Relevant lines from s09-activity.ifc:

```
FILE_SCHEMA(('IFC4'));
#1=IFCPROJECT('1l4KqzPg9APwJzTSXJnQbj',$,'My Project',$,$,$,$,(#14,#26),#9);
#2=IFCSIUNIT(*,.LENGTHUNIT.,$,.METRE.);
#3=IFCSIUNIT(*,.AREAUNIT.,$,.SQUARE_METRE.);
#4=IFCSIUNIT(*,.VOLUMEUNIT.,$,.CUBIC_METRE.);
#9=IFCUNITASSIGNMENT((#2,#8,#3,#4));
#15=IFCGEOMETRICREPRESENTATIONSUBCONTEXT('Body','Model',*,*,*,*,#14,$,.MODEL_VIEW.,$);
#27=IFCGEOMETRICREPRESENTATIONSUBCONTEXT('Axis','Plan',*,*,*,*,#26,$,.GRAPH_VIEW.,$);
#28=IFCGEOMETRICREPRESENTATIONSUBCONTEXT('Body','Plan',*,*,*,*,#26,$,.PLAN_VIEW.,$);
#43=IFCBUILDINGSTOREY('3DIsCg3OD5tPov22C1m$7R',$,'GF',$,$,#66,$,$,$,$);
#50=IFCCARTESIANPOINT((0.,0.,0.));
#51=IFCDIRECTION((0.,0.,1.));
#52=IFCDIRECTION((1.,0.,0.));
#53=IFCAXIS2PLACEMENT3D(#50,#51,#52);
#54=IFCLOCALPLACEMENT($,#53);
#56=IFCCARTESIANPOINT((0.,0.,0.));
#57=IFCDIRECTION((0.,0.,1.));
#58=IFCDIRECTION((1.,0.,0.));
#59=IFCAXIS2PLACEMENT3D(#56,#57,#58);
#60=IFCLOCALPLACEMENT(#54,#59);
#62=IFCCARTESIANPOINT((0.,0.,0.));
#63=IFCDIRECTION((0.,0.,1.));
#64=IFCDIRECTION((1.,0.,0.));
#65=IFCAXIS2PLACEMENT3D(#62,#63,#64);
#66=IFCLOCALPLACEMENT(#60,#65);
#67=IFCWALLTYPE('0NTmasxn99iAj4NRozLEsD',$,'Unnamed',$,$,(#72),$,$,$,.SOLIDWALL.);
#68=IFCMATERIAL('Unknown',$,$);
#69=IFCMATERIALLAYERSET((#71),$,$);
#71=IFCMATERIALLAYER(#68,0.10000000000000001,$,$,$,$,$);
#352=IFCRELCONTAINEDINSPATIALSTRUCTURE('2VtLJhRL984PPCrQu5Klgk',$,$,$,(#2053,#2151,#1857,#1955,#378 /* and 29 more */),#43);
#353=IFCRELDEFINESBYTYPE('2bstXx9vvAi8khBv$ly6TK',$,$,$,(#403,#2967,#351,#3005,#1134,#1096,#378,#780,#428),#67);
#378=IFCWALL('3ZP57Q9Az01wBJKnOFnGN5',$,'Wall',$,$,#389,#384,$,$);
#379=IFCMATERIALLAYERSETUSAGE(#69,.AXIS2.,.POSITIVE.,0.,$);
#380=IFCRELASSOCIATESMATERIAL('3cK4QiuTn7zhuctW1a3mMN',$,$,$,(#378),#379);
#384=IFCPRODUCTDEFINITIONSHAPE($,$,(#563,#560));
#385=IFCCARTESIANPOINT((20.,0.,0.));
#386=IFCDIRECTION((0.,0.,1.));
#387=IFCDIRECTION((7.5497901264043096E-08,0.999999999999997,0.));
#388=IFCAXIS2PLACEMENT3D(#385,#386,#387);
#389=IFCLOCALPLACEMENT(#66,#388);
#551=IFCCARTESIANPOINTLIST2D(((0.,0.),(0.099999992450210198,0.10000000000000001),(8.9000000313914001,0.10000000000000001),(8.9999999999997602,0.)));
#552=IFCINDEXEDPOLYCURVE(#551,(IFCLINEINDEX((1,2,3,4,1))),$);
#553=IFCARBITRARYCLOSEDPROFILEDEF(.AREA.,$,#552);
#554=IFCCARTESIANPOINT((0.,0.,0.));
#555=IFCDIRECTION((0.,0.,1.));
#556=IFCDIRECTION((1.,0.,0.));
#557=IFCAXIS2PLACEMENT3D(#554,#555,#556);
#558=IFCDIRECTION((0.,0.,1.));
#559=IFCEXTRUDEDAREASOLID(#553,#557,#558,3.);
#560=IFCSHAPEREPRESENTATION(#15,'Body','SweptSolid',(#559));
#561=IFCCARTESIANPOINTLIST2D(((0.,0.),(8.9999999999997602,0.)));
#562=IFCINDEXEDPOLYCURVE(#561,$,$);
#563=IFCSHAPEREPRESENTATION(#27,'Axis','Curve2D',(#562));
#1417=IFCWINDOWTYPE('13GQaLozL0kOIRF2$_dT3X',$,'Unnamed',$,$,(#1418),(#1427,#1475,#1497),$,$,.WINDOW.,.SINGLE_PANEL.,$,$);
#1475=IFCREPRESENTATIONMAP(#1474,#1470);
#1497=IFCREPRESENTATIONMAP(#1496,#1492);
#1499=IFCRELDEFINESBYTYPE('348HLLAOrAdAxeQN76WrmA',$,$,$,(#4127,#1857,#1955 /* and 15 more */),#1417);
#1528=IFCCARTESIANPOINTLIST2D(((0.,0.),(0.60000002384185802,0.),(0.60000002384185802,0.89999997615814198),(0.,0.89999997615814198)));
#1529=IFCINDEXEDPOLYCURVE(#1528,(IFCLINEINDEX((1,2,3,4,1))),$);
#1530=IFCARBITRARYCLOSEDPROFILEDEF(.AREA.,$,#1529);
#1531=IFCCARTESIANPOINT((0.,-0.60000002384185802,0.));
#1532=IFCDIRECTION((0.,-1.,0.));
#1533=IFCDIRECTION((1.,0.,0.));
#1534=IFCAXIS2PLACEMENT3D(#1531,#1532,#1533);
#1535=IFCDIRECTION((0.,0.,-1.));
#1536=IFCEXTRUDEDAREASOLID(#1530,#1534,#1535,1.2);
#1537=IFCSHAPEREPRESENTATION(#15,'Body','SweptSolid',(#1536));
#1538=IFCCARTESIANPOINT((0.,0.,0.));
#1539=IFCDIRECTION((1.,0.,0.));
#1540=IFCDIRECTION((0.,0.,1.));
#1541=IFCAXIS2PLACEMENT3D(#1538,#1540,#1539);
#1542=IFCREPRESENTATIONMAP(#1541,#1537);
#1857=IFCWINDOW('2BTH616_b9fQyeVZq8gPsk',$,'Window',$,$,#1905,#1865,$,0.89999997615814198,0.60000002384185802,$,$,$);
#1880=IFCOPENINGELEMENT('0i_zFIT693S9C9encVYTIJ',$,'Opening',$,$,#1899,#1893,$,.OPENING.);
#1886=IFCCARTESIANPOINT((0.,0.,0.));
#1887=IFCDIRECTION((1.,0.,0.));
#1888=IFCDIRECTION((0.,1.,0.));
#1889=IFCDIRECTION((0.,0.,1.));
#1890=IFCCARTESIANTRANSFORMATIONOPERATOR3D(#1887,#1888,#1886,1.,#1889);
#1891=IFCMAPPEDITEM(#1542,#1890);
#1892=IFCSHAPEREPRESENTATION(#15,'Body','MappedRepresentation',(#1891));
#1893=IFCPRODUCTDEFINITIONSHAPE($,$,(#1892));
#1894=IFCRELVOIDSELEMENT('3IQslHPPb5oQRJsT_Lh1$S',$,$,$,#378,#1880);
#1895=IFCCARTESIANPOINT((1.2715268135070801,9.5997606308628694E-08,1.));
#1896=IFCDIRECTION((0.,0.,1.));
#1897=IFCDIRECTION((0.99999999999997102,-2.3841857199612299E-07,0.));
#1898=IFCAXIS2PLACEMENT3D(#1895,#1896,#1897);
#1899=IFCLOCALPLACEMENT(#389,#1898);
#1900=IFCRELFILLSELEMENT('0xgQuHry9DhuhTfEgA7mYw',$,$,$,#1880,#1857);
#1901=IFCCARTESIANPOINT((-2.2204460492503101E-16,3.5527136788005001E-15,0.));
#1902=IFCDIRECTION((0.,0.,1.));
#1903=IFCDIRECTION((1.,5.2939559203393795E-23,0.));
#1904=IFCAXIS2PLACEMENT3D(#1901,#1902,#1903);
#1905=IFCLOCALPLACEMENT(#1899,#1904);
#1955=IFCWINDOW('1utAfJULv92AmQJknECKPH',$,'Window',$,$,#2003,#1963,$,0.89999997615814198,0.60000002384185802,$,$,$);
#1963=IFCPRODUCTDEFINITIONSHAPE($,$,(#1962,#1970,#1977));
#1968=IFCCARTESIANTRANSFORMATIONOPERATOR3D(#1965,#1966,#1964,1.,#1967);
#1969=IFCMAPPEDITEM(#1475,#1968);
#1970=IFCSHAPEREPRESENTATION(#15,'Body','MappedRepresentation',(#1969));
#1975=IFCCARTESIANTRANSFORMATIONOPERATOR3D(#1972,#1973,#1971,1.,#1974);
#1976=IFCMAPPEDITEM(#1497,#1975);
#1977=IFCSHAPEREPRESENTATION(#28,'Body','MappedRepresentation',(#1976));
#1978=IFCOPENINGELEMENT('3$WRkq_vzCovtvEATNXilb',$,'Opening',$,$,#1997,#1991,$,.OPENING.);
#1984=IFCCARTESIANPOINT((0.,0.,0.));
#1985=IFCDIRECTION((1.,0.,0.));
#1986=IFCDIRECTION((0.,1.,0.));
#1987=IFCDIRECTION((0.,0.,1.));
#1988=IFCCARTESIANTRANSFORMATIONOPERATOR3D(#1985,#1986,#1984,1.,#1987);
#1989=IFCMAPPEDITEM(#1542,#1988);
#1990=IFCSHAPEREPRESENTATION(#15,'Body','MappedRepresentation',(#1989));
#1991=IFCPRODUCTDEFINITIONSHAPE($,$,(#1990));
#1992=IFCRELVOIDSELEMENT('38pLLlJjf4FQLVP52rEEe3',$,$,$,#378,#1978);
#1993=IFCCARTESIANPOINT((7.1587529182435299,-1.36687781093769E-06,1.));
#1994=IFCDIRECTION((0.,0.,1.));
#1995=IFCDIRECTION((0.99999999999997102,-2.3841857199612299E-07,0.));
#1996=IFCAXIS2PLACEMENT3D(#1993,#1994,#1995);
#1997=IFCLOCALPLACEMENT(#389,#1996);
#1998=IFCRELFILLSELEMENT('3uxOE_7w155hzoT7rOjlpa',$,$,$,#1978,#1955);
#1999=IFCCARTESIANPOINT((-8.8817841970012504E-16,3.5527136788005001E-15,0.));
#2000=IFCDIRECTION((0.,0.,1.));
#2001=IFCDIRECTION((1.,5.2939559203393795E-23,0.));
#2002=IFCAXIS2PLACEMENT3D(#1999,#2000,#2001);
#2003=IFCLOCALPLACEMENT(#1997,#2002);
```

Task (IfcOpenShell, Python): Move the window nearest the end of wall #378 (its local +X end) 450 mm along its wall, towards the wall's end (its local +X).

```python
import ifcopenshell
import ifcopenshell.api.geometry
import ifcopenshell.util.placement

model = ifcopenshell.open("s09-activity.ifc")

window = model.by_guid("1utAfJULv92AmQJknECKPH")
opening = window.FillsVoids[0].RelatingOpeningElement
wall = opening.VoidsElements[0].RelatingBuildingElement

wall_matrix = ifcopenshell.util.placement.get_local_placement(wall.ObjectPlacement)
shift = wall_matrix[:3, 0] * 0.45
before = ifcopenshell.util.placement.get_local_placement(window.ObjectPlacement)[:3, 3].copy()

# The window is placed relative to its opening, so it follows when the opening moves.
matrix = ifcopenshell.util.placement.get_local_placement(opening.ObjectPlacement)
matrix[:3, 3] += shift
ifcopenshell.api.geometry.edit_object_placement(
    model, product=opening, matrix=matrix, is_si=False, should_transform_children=True
)

after = ifcopenshell.util.placement.get_local_placement(window.ObjectPlacement)[:3, 3]
print("window moved by", (after - before).round(3) + 0.0)

model.write("s09-activity_rev.ifc")
```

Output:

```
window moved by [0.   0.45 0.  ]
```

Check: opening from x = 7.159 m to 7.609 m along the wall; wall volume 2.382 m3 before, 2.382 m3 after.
